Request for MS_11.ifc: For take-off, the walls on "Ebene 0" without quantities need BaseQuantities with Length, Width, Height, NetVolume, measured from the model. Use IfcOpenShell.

First a look at what the model holds.

```python
import ifcopenshell
import ifcopenshell.util.element
import ifcopenshell.util.unit

model = ifcopenshell.open("MS_11.ifc")
print(model.schema)
for unit_type in ("LENGTHUNIT", "AREAUNIT", "VOLUMEUNIT"):
    print(unit_type, ifcopenshell.util.unit.calculate_unit_scale(model, unit_type))
storey = next(s for s in model.by_type("IfcBuildingStorey") if s.Name == "Ebene 0")
walls = [e for e in ifcopenshell.util.element.get_decomposition(storey) if e.is_a("IfcWall")]
for e in sorted(walls, key=lambda e: e.id()):
    print(e.id(), e.is_a(), e.Name, list(ifcopenshell.util.element.get_psets(e, qtos_only=True)), sep=" | ")
```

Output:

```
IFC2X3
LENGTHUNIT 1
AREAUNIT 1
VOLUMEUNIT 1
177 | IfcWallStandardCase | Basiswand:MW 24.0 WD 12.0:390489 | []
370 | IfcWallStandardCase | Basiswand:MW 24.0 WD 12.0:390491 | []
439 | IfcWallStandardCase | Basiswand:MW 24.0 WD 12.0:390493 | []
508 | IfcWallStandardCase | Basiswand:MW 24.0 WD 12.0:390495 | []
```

```python
import ifcopenshell
import ifcopenshell.api.pset
import ifcopenshell.geom
import ifcopenshell.util.element
import ifcopenshell.util.shape
import ifcopenshell.util.unit

model = ifcopenshell.open("MS_11.ifc")
unit_scale = ifcopenshell.util.unit.calculate_unit_scale(model)
volume_scale = ifcopenshell.util.unit.calculate_unit_scale(model, "VOLUMEUNIT")
settings = ifcopenshell.geom.settings()

storey = next(s for s in model.by_type("IfcBuildingStorey") if s.Name == "Ebene 0")
walls = [e for e in ifcopenshell.util.element.get_decomposition(storey) if e.is_a("IfcWall")]

for e in sorted(walls, key=lambda e: e.id()):
    if ifcopenshell.util.element.get_psets(e, qtos_only=True, should_inherit=False):
        continue
    # Geometry comes back in metres, in the element's own axes.
    shape = ifcopenshell.geom.create_shape(settings, e)
    values = {
        "Length": ifcopenshell.util.shape.get_x(shape.geometry) / unit_scale,
        "Width": ifcopenshell.util.shape.get_y(shape.geometry) / unit_scale,
        "Height": ifcopenshell.util.shape.get_z(shape.geometry) / unit_scale,
        "NetVolume": ifcopenshell.util.shape.get_volume(shape.geometry) / volume_scale,
    }
    qto = ifcopenshell.api.pset.add_qto(model, product=e, name="BaseQuantities")
    ifcopenshell.api.pset.edit_qto(model, qto=qto, properties=values)
    print(e.id(), {k: round(v, 3) for k, v in values.items()})

model.write("MS_11_edited.ifc")
```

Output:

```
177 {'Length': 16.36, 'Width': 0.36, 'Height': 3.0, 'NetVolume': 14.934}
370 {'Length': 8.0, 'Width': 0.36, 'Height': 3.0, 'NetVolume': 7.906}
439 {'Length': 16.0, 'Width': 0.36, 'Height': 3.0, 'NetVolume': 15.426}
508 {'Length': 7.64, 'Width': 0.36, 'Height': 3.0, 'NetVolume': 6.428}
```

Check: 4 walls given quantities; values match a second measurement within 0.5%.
